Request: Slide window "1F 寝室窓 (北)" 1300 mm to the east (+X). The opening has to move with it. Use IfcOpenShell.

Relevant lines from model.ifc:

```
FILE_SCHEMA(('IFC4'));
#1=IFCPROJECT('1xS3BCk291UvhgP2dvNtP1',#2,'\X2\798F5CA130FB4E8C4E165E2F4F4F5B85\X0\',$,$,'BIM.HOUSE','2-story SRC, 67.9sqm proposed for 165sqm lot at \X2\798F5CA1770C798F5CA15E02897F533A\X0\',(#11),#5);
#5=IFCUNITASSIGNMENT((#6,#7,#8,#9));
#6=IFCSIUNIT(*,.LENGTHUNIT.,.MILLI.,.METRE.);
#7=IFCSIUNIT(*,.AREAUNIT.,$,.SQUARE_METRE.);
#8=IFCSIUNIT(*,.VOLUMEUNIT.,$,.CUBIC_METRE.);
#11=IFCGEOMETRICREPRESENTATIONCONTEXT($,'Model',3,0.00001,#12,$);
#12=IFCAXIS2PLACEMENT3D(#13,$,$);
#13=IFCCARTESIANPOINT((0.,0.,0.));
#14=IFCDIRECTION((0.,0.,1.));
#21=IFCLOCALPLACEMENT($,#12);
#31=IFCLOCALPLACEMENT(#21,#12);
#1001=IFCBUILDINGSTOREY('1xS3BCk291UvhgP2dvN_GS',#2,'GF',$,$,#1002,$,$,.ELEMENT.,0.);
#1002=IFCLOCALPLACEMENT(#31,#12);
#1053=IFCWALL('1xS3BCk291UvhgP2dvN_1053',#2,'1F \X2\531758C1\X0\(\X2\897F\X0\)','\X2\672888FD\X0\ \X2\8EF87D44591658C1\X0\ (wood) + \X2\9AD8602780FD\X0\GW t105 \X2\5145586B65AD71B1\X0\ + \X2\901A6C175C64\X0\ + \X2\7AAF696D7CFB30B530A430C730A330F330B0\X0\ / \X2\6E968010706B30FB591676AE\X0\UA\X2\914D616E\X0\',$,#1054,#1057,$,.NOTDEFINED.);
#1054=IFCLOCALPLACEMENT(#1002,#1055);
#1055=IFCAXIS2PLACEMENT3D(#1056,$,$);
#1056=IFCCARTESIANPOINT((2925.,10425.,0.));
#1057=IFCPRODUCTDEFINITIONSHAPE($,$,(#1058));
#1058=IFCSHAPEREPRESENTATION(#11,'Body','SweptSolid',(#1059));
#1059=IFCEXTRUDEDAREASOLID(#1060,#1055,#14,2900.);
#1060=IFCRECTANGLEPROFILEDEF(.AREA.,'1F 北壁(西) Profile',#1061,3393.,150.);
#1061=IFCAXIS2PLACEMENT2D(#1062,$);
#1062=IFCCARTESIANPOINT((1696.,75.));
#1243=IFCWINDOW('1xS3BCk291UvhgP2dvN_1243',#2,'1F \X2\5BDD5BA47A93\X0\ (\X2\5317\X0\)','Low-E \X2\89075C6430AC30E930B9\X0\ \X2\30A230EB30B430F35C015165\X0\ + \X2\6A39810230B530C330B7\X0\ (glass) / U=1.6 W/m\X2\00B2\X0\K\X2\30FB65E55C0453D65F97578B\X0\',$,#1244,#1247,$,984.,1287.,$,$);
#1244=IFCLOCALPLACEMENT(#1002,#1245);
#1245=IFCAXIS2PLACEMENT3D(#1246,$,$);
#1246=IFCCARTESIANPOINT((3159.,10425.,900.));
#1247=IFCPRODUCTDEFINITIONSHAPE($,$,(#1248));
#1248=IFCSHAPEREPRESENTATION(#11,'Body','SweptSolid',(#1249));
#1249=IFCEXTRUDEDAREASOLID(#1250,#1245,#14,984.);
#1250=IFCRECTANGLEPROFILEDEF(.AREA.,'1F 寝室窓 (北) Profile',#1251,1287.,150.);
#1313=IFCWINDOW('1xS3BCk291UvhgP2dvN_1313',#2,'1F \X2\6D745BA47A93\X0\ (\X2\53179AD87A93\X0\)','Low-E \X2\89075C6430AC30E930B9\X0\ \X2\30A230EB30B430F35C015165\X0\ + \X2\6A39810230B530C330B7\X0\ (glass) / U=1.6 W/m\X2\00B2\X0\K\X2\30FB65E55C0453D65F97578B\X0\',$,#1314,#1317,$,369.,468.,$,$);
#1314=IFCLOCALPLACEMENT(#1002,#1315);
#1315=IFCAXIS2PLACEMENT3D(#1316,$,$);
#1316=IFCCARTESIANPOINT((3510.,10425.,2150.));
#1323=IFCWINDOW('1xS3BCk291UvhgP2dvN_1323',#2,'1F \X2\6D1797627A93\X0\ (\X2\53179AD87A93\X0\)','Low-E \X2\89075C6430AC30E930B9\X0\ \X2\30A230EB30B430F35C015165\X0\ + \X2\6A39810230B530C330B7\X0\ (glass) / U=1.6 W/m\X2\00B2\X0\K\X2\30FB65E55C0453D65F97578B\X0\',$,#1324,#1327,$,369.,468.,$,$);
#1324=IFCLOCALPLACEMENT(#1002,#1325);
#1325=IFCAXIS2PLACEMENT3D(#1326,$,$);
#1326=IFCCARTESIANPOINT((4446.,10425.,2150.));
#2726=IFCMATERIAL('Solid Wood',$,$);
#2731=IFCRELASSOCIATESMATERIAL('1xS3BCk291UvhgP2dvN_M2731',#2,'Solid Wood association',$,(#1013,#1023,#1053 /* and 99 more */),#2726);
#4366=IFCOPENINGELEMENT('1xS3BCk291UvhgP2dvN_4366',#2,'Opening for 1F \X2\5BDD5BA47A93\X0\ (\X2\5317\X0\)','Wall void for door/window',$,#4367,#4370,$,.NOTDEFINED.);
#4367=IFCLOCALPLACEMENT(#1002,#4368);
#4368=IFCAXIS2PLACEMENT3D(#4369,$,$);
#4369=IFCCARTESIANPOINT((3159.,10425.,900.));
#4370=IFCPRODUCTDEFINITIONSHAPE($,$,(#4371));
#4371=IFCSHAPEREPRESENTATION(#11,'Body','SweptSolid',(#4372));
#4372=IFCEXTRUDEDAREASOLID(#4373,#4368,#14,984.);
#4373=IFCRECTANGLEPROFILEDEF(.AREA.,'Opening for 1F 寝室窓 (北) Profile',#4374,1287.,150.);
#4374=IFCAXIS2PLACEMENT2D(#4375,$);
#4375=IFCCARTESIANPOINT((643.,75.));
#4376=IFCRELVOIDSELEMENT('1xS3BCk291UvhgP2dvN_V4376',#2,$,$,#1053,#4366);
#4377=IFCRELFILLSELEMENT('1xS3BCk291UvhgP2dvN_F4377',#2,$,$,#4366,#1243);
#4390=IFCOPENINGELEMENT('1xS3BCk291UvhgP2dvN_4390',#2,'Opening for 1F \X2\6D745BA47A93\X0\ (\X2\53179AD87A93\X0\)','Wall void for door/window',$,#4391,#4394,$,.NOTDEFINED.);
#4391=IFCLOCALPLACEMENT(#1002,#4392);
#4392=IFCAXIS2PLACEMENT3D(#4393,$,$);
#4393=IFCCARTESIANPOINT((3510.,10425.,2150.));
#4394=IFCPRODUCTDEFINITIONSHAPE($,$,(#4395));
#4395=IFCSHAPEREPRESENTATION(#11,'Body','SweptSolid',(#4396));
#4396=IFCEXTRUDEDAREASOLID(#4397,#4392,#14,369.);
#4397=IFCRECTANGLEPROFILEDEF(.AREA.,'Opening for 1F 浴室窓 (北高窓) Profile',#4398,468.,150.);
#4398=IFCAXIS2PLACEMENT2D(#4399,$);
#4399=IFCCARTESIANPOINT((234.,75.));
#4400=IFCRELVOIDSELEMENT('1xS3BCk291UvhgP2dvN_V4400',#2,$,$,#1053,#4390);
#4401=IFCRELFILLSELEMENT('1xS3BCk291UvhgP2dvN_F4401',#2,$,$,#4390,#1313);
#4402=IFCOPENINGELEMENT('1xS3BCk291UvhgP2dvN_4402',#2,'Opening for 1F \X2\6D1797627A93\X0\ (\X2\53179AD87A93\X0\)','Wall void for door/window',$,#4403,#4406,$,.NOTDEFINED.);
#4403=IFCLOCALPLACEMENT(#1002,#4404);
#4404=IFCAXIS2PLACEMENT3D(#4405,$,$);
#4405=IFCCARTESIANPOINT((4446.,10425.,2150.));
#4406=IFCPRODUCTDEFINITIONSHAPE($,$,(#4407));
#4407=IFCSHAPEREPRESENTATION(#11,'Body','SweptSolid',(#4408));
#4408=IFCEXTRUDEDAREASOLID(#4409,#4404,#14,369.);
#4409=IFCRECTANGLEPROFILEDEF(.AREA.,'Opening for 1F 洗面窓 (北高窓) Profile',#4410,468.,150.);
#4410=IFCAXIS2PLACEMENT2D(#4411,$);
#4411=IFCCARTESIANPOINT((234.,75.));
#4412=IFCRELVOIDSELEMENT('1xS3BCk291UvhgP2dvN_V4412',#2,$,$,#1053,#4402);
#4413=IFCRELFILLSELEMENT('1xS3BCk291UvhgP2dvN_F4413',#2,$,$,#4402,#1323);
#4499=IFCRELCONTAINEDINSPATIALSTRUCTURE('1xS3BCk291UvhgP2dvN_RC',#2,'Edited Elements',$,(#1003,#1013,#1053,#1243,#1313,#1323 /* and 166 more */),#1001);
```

```python
import ifcopenshell
import ifcopenshell.api.geometry
import ifcopenshell.util.placement
import ifcopenshell.util.unit

model = ifcopenshell.open("model.ifc")
unit_scale = ifcopenshell.util.unit.calculate_unit_scale(model)

window = model.by_guid("1xS3BCk291UvhgP2dvN_1243")
opening = window.FillsVoids[0].RelatingOpeningElement
wall = opening.VoidsElements[0].RelatingBuildingElement

wall_matrix = ifcopenshell.util.placement.get_local_placement(wall.ObjectPlacement)
shift = wall_matrix[:3, 0] * 1.3 / unit_scale
before = ifcopenshell.util.placement.get_local_placement(window.ObjectPlacement)[:3, 3].copy()

# The window is not placed relative to its opening, so move both.
for product in (opening, window):
    matrix = ifcopenshell.util.placement.get_local_placement(product.ObjectPlacement)
    matrix[:3, 3] += shift
    ifcopenshell.api.geometry.edit_object_placement(model, product=product, matrix=matrix, is_si=False)

after = ifcopenshell.util.placement.get_local_placement(window.ObjectPlacement)[:3, 3]
print("window moved by", (after - before).round(3) + 0.0)

model.write("model-out.ifc")
```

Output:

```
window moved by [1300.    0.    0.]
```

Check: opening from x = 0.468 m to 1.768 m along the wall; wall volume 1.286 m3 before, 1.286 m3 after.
